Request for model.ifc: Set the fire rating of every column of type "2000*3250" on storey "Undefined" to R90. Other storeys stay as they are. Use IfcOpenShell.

First a look at what the model holds.

```python
import ifcopenshell
import ifcopenshell.util.element

model = ifcopenshell.open("model.ifc")
print(model.schema)
storey = next(s for s in model.by_type("IfcBuildingStorey") if s.Name == "Undefined")
columns = [e for e in ifcopenshell.util.element.get_decomposition(storey) if e.is_a("IfcColumn")]
seen = {}
for e in columns:
    element_type = ifcopenshell.util.element.get_type(e)
    key = (element_type.Name if element_type != e and element_type else None, ifcopenshell.util.element.get_pset(e, "Pset_ColumnCommon", "FireRating"))
    seen[key] = seen.get(key, 0) + 1
for (name, value), count in sorted(seen.items(), key=str):
    print(count, "x", name, "|", value)
```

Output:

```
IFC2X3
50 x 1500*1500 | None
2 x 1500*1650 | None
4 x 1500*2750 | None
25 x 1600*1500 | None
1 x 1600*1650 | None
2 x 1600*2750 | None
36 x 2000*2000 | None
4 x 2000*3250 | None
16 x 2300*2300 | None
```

```python
import ifcopenshell
import ifcopenshell.api.pset
import ifcopenshell.util.element

model = ifcopenshell.open("model.ifc")

storey = next(s for s in model.by_type("IfcBuildingStorey") if s.Name == "Undefined")
columns = [e for e in ifcopenshell.util.element.get_decomposition(storey) if e.is_a("IfcColumn")]

count = 0
for e in columns:
    element_type = ifcopenshell.util.element.get_type(e)
    if element_type in (None, e) or element_type.Name != "2000*3250":
        continue
    found = ifcopenshell.util.element.get_pset(e, "Pset_ColumnCommon", should_inherit=False)
    if found:
        pset = model.by_id(found["id"])
        if len(ifcopenshell.util.element.get_elements_by_pset(pset)) > 1:
            pset = ifcopenshell.api.pset.unshare_pset(model, products=[e], pset=pset)[0]
    else:
        pset = ifcopenshell.api.pset.add_pset(model, product=e, name="Pset_ColumnCommon")
    ifcopenshell.api.pset.edit_pset(model, pset=pset, properties={"FireRating": "R90"})
    count += 1

print(count, "columns updated")

model.write("model_edited.ifc")
```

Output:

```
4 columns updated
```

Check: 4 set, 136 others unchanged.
